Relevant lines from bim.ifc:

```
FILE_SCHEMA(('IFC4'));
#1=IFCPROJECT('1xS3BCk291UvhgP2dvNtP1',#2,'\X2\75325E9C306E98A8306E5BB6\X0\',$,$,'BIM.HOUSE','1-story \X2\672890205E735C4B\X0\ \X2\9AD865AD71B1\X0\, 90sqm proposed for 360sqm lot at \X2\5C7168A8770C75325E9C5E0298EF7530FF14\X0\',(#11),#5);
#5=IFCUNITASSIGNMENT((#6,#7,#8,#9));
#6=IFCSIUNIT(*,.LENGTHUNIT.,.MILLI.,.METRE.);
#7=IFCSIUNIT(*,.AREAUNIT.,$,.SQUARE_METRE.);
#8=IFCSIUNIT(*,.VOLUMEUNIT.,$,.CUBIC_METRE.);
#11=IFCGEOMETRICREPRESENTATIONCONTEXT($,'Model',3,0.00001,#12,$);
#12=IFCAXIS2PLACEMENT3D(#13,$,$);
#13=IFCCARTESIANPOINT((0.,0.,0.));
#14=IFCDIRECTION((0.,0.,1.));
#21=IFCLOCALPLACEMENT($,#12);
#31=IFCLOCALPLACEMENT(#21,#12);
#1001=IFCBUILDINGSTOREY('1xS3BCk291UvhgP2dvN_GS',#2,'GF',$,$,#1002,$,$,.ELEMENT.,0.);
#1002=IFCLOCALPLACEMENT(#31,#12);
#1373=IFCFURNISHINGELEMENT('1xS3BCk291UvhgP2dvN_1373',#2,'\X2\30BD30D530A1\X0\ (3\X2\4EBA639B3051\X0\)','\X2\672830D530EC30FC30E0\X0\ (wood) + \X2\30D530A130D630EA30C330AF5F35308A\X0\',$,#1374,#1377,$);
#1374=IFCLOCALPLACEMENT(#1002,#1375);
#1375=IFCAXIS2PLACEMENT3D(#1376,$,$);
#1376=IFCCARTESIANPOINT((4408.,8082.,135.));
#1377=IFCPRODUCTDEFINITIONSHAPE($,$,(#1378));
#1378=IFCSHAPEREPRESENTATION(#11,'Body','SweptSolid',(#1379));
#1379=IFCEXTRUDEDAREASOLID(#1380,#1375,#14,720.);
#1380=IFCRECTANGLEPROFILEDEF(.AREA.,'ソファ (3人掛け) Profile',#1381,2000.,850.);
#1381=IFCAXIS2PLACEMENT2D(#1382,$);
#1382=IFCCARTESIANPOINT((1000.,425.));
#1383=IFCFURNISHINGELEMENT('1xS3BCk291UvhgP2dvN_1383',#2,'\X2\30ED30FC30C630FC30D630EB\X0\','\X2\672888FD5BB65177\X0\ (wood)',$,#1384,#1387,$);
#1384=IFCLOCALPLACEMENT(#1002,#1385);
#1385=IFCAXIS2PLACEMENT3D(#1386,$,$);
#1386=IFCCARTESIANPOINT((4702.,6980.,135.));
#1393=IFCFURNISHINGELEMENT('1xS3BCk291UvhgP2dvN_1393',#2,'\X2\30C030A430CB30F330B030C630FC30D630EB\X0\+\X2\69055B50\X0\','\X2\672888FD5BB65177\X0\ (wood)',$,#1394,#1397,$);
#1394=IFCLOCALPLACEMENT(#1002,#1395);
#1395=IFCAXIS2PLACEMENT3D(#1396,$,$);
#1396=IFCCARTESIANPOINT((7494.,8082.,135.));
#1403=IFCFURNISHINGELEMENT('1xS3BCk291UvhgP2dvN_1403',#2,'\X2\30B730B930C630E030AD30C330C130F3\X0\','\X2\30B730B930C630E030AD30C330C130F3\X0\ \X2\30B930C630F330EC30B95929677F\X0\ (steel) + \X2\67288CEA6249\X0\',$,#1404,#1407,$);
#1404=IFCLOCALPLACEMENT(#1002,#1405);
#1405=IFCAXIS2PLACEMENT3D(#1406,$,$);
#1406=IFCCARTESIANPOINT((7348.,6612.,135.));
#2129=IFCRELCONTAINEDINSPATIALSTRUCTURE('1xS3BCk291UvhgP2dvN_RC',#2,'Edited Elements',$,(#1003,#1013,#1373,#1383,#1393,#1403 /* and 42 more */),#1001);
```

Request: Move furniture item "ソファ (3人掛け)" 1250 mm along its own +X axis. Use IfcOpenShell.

```python
import ifcopenshell
import ifcopenshell.api.geometry
import ifcopenshell.util.placement

model = ifcopenshell.open("bim.ifc")

item = model.by_id(1373)
matrix = ifcopenshell.util.placement.get_local_placement(item.ObjectPlacement)
matrix[:3, 3] += matrix[:3, 0] * 1250.0
ifcopenshell.api.geometry.edit_object_placement(model, product=item, matrix=matrix, is_si=False)

print(ifcopenshell.util.placement.get_local_placement(item.ObjectPlacement).round(3) + 0.0)

model.write("bim_rev.ifc")
```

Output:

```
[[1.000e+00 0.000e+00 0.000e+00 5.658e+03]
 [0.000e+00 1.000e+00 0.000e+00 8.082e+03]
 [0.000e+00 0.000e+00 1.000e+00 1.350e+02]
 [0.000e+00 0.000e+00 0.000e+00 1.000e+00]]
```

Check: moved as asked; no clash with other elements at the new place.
